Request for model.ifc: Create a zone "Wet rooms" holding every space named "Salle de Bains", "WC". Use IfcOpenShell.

First a look at what the model holds.

```python
import ifcopenshell

model = ifcopenshell.open("model.ifc")
print(model.schema)
seen = {}
for space in model.by_type("IfcSpace"):
    seen[space.LongName] = seen.get(space.LongName, 0) + 1
for name, count in sorted(seen.items(), key=str):
    print(count, "x", name)
print("zones:", [z.Name for z in model.by_type("IfcZone")][:20])
```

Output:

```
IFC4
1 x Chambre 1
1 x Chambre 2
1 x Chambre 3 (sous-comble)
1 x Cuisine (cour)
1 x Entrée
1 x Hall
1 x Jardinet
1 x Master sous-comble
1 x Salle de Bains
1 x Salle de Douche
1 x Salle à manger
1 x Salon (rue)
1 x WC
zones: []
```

```python
import ifcopenshell
import ifcopenshell.api.group
import ifcopenshell.api.root

model = ifcopenshell.open("model.ifc")

names = {"Salle de Bains", "WC"}
spaces = [s for s in model.by_type("IfcSpace") if s.LongName in names]

zone = ifcopenshell.api.root.create_entity(model, ifc_class="IfcZone", name="Wet rooms")
ifcopenshell.api.group.assign_group(model, products=spaces, group=zone)
print(len(spaces), "spaces in", zone.Name)

model.write("model_rev.ifc")
```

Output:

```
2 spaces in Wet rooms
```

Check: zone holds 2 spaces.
